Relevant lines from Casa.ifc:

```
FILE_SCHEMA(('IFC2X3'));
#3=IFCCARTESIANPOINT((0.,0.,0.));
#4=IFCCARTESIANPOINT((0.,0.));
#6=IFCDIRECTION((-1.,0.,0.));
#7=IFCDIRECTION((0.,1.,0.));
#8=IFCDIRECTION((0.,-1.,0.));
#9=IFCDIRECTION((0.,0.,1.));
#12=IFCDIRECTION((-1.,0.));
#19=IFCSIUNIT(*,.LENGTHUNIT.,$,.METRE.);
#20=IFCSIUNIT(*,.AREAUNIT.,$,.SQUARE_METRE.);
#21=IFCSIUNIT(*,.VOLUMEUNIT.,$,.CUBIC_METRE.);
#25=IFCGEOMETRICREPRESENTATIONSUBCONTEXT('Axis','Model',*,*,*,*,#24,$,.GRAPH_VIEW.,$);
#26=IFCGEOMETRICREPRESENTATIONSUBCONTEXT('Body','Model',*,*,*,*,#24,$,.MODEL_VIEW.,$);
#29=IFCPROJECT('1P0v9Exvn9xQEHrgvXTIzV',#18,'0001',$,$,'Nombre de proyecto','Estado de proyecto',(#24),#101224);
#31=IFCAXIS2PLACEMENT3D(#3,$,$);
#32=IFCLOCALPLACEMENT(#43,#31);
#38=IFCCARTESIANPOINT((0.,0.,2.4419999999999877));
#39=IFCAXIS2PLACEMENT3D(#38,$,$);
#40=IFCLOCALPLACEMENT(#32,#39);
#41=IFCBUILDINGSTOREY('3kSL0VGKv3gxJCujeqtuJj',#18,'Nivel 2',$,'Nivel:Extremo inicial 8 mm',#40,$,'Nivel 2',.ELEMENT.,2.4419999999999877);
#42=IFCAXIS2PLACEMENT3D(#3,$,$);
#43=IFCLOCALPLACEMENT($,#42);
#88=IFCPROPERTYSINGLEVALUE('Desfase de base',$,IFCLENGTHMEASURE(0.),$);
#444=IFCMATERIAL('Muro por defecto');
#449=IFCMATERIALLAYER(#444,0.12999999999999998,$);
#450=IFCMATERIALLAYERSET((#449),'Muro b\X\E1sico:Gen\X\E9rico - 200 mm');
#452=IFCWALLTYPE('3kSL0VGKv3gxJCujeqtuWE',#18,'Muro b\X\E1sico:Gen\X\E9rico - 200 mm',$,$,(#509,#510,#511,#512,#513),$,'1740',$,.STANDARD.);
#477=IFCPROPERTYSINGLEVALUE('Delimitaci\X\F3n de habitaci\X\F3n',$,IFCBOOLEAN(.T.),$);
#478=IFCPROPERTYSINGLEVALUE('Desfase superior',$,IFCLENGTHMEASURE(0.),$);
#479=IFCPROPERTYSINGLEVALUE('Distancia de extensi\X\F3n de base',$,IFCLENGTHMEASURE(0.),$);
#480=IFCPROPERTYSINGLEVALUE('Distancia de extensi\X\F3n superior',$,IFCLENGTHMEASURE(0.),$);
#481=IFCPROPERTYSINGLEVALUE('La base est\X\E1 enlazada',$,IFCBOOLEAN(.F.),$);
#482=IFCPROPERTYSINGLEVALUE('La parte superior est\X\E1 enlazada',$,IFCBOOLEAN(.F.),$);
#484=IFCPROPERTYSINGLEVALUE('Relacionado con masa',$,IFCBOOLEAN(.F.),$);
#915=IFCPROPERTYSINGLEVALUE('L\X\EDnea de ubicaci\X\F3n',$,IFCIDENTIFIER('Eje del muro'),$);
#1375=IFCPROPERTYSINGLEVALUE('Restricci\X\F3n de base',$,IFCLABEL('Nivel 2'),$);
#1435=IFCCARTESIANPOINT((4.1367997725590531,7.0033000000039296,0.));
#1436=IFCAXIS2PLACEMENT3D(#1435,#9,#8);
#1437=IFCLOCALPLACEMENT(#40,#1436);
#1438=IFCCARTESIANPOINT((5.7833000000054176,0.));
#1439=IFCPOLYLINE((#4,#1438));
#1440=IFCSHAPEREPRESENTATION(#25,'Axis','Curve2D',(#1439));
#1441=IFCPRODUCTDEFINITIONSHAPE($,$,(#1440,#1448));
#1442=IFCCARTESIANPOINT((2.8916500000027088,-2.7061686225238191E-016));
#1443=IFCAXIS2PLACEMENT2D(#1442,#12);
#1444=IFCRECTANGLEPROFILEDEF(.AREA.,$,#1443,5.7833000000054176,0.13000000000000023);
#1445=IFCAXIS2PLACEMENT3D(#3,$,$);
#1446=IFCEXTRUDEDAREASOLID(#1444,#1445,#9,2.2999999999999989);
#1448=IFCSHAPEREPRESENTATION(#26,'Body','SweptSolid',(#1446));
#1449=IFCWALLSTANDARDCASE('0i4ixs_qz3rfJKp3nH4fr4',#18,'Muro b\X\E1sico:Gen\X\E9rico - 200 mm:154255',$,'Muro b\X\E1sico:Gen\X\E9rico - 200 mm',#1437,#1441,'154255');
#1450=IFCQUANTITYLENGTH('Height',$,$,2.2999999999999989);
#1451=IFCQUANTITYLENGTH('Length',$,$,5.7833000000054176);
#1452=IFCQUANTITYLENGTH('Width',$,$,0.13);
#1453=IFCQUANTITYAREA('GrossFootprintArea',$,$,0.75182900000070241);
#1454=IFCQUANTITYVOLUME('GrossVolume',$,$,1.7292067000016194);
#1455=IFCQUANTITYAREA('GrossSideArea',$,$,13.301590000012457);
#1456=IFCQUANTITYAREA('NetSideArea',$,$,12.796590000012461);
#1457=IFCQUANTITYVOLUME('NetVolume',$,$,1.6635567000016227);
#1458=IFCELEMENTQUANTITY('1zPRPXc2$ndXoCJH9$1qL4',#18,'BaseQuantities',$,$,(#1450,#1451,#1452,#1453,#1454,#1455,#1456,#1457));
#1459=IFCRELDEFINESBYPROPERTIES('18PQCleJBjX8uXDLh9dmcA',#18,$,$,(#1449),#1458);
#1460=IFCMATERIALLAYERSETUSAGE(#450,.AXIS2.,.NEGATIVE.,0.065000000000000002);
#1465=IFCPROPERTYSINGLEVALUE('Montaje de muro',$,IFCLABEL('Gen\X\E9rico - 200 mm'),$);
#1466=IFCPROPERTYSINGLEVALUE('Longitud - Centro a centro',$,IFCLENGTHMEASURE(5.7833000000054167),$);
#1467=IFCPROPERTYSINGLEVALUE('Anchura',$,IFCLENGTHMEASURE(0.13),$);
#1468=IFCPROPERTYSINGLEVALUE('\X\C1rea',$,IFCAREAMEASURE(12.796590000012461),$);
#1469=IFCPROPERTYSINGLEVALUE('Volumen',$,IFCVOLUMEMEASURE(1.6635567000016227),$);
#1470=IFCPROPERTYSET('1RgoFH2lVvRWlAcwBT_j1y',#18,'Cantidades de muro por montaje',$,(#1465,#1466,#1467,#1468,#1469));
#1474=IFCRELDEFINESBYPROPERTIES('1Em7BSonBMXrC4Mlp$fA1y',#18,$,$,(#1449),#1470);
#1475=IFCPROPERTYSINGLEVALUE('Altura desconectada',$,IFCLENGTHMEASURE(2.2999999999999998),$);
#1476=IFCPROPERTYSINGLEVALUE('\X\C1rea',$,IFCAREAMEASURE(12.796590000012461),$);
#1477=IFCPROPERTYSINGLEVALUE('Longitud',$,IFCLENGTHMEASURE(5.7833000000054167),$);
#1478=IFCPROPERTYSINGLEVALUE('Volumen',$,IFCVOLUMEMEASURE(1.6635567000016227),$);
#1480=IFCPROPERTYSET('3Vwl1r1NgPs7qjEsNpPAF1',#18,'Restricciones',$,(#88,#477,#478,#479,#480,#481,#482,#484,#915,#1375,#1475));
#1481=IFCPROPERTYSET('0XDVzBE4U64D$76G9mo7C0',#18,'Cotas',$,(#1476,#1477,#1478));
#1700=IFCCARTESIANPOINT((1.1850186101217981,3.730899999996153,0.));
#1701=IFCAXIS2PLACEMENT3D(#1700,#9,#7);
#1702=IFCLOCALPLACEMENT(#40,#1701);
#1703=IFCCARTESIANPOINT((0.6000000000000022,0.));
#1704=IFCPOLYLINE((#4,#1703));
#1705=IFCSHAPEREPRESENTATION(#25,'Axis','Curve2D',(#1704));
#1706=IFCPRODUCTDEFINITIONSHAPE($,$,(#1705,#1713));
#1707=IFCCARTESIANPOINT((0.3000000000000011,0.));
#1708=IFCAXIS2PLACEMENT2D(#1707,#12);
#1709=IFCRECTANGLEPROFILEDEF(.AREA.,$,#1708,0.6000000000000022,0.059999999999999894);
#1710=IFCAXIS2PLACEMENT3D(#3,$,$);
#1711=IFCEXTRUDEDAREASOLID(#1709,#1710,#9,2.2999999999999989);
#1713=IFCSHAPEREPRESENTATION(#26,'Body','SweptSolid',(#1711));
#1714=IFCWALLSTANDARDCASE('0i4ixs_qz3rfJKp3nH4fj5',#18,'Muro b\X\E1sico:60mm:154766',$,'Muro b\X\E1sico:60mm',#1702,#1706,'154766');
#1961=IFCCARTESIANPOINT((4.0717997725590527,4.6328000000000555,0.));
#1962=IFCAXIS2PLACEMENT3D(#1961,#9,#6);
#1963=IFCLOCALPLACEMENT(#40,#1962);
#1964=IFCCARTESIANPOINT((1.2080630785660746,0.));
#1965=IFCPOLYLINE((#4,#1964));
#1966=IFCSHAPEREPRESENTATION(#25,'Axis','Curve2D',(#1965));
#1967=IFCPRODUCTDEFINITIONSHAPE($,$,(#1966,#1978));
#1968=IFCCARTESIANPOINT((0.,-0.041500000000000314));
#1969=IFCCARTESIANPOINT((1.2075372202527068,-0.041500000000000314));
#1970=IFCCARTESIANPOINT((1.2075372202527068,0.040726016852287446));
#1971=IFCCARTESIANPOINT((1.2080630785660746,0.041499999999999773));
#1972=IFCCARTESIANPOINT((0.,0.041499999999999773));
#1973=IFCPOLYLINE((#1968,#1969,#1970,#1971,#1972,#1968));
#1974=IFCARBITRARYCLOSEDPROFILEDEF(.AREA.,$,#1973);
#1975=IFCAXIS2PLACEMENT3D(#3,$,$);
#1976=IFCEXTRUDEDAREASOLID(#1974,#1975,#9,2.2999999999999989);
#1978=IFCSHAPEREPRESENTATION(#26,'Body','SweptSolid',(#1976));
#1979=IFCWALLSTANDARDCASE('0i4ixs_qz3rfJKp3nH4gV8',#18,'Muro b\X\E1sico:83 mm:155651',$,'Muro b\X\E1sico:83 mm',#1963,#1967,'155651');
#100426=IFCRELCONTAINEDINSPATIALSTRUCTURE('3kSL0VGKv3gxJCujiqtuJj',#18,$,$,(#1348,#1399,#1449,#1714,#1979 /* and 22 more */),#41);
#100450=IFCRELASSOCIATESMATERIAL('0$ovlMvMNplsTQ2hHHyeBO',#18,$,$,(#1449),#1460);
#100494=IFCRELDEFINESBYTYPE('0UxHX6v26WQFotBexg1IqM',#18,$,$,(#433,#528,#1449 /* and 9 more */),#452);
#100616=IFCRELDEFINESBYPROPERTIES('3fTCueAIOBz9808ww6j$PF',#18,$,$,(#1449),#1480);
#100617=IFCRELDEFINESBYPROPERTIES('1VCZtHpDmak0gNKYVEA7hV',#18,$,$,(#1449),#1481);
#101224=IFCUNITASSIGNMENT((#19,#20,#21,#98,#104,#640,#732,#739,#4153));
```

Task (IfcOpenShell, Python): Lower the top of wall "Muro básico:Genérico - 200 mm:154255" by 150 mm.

```python
import ifcopenshell
import ifcopenshell.api.pset
import ifcopenshell.geom
import ifcopenshell.util.element
import ifcopenshell.util.representation
import ifcopenshell.util.shape
import ifcopenshell.util.unit

model = ifcopenshell.open("Casa.ifc")
unit_scale = ifcopenshell.util.unit.calculate_unit_scale(model)
area_scale = ifcopenshell.util.unit.calculate_unit_scale(model, "AREAUNIT")
volume_scale = ifcopenshell.util.unit.calculate_unit_scale(model, "VOLUMEUNIT")
settings = ifcopenshell.geom.settings()


def volume(element):
    """Net volume in cubic metres, openings subtracted."""
    shape = ifcopenshell.geom.create_shape(settings, element)
    return ifcopenshell.util.shape.get_volume(shape.geometry)


wall = model.by_guid("0i4ixs_qz3rfJKp3nH4fr4")
before = volume(wall)

body = ifcopenshell.util.representation.get_representation(wall, "Model", "Body")
solid = body.Items[0]
old_height = solid.Depth
solid.Depth -= 0.15 / unit_scale
after = volume(wall)
thickness = 0.13  # wall thickness in metres

# Update the stored height, areas and volumes.
qto = model.by_id(ifcopenshell.util.element.get_pset(wall, "BaseQuantities", should_inherit=False)["id"])
ifcopenshell.api.pset.edit_qto(model, qto=qto, properties={
    "Height": solid.Depth,
    "GrossVolume": ifcopenshell.util.element.get_pset(wall, "BaseQuantities", "GrossVolume") * solid.Depth / old_height,
    "GrossSideArea": ifcopenshell.util.element.get_pset(wall, "BaseQuantities", "GrossSideArea") * solid.Depth / old_height,
    "NetSideArea": after / thickness / area_scale,
    "NetVolume": after / volume_scale,
})
pset = model.by_id(ifcopenshell.util.element.get_pset(wall, "Cantidades de muro por montaje", should_inherit=False)["id"])
ifcopenshell.api.pset.edit_pset(model, pset=pset, properties={
    "Área": model.create_entity("IfcAreaMeasure", after / thickness / area_scale),
    "Volumen": model.create_entity("IfcVolumeMeasure", after / volume_scale),
})
pset = model.by_id(ifcopenshell.util.element.get_pset(wall, "Restricciones", should_inherit=False)["id"])
ifcopenshell.api.pset.edit_pset(model, pset=pset, properties={
    "Altura desconectada": model.create_entity("IfcLengthMeasure", solid.Depth),
})
pset = model.by_id(ifcopenshell.util.element.get_pset(wall, "Cotas", should_inherit=False)["id"])
ifcopenshell.api.pset.edit_pset(model, pset=pset, properties={
    "Área": model.create_entity("IfcAreaMeasure", after / thickness / area_scale),
    "Volumen": model.create_entity("IfcVolumeMeasure", after / volume_scale),
})

print(f"height {old_height:g} -> {solid.Depth:g}, volume {before:.3f} -> {after:.3f} m3")

model.write("Casa_updated.ifc")
```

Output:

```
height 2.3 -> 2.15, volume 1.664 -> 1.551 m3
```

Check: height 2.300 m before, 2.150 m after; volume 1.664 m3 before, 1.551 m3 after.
